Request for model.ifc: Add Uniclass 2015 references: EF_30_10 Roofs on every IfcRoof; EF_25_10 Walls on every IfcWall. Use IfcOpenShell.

First a look at what the model holds.

```python
import ifcopenshell

model = ifcopenshell.open("model.ifc")
print(model.schema)
print("classifications:", [c.Name for c in model.by_type("IfcClassification")])
for ifc_class in ("IfcDoor", "IfcRoof", "IfcStair", "IfcWall", "IfcWindow"):
    print(ifc_class, len(model.by_type(ifc_class)))
```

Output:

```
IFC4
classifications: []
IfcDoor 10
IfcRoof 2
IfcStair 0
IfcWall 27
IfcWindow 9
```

```python
import ifcopenshell
import ifcopenshell.api.classification

model = ifcopenshell.open("model.ifc")

system = ifcopenshell.api.classification.add_classification(model, classification="Uniclass 2015")

codes = {
    "IfcRoof": ("EF_30_10", "Roofs"),
    "IfcWall": ("EF_25_10", "Walls"),
}
for ifc_class, (code, name) in codes.items():
    products = model.by_type(ifc_class)
    ifcopenshell.api.classification.add_reference(
        model, products=products, classification=system, identification=code, name=name
    )
    print(code, len(products))

model.write("model_rev.ifc")
```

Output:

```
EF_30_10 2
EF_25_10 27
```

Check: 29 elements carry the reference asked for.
